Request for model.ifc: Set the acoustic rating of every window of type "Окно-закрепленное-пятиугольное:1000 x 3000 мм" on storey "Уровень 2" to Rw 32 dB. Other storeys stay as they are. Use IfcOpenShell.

First a look at what the model holds.

```python
import ifcopenshell
import ifcopenshell.util.element

model = ifcopenshell.open("model.ifc")
print(model.schema)
storey = next(s for s in model.by_type("IfcBuildingStorey") if s.Name == "Уровень 2")
windows = [e for e in ifcopenshell.util.element.get_decomposition(storey) if e.is_a("IfcWindow")]
seen = {}
for e in windows:
    element_type = ifcopenshell.util.element.get_type(e)
    key = (element_type.Name if element_type != e and element_type else None, ifcopenshell.util.element.get_pset(e, "Pset_WindowCommon", "AcousticRating"))
    seen[key] = seen.get(key, 0) + 1
for (name, value), count in sorted(seen.items(), key=str):
    print(count, "x", name, "|", value)
```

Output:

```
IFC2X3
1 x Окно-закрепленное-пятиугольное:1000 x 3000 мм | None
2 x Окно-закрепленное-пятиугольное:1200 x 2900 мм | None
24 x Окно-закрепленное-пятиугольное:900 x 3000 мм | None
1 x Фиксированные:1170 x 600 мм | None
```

```python
import ifcopenshell
import ifcopenshell.api.pset
import ifcopenshell.util.element

model = ifcopenshell.open("model.ifc")

storey = next(s for s in model.by_type("IfcBuildingStorey") if s.Name == "Уровень 2")
windows = [e for e in ifcopenshell.util.element.get_decomposition(storey) if e.is_a("IfcWindow")]

count = 0
for e in windows:
    element_type = ifcopenshell.util.element.get_type(e)
    if element_type in (None, e) or element_type.Name != "Окно-закрепленное-пятиугольное:1000 x 3000 мм":
        continue
    # add_pset returns the element's existing set when there is one.
    pset = ifcopenshell.api.pset.add_pset(model, product=e, name="Pset_WindowCommon")
    ifcopenshell.api.pset.edit_pset(model, pset=pset, properties={"AcousticRating": "Rw 32 dB"})
    count += 1

print(count, "windows updated")

model.write("model-out.ifc")
```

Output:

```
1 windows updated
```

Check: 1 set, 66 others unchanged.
